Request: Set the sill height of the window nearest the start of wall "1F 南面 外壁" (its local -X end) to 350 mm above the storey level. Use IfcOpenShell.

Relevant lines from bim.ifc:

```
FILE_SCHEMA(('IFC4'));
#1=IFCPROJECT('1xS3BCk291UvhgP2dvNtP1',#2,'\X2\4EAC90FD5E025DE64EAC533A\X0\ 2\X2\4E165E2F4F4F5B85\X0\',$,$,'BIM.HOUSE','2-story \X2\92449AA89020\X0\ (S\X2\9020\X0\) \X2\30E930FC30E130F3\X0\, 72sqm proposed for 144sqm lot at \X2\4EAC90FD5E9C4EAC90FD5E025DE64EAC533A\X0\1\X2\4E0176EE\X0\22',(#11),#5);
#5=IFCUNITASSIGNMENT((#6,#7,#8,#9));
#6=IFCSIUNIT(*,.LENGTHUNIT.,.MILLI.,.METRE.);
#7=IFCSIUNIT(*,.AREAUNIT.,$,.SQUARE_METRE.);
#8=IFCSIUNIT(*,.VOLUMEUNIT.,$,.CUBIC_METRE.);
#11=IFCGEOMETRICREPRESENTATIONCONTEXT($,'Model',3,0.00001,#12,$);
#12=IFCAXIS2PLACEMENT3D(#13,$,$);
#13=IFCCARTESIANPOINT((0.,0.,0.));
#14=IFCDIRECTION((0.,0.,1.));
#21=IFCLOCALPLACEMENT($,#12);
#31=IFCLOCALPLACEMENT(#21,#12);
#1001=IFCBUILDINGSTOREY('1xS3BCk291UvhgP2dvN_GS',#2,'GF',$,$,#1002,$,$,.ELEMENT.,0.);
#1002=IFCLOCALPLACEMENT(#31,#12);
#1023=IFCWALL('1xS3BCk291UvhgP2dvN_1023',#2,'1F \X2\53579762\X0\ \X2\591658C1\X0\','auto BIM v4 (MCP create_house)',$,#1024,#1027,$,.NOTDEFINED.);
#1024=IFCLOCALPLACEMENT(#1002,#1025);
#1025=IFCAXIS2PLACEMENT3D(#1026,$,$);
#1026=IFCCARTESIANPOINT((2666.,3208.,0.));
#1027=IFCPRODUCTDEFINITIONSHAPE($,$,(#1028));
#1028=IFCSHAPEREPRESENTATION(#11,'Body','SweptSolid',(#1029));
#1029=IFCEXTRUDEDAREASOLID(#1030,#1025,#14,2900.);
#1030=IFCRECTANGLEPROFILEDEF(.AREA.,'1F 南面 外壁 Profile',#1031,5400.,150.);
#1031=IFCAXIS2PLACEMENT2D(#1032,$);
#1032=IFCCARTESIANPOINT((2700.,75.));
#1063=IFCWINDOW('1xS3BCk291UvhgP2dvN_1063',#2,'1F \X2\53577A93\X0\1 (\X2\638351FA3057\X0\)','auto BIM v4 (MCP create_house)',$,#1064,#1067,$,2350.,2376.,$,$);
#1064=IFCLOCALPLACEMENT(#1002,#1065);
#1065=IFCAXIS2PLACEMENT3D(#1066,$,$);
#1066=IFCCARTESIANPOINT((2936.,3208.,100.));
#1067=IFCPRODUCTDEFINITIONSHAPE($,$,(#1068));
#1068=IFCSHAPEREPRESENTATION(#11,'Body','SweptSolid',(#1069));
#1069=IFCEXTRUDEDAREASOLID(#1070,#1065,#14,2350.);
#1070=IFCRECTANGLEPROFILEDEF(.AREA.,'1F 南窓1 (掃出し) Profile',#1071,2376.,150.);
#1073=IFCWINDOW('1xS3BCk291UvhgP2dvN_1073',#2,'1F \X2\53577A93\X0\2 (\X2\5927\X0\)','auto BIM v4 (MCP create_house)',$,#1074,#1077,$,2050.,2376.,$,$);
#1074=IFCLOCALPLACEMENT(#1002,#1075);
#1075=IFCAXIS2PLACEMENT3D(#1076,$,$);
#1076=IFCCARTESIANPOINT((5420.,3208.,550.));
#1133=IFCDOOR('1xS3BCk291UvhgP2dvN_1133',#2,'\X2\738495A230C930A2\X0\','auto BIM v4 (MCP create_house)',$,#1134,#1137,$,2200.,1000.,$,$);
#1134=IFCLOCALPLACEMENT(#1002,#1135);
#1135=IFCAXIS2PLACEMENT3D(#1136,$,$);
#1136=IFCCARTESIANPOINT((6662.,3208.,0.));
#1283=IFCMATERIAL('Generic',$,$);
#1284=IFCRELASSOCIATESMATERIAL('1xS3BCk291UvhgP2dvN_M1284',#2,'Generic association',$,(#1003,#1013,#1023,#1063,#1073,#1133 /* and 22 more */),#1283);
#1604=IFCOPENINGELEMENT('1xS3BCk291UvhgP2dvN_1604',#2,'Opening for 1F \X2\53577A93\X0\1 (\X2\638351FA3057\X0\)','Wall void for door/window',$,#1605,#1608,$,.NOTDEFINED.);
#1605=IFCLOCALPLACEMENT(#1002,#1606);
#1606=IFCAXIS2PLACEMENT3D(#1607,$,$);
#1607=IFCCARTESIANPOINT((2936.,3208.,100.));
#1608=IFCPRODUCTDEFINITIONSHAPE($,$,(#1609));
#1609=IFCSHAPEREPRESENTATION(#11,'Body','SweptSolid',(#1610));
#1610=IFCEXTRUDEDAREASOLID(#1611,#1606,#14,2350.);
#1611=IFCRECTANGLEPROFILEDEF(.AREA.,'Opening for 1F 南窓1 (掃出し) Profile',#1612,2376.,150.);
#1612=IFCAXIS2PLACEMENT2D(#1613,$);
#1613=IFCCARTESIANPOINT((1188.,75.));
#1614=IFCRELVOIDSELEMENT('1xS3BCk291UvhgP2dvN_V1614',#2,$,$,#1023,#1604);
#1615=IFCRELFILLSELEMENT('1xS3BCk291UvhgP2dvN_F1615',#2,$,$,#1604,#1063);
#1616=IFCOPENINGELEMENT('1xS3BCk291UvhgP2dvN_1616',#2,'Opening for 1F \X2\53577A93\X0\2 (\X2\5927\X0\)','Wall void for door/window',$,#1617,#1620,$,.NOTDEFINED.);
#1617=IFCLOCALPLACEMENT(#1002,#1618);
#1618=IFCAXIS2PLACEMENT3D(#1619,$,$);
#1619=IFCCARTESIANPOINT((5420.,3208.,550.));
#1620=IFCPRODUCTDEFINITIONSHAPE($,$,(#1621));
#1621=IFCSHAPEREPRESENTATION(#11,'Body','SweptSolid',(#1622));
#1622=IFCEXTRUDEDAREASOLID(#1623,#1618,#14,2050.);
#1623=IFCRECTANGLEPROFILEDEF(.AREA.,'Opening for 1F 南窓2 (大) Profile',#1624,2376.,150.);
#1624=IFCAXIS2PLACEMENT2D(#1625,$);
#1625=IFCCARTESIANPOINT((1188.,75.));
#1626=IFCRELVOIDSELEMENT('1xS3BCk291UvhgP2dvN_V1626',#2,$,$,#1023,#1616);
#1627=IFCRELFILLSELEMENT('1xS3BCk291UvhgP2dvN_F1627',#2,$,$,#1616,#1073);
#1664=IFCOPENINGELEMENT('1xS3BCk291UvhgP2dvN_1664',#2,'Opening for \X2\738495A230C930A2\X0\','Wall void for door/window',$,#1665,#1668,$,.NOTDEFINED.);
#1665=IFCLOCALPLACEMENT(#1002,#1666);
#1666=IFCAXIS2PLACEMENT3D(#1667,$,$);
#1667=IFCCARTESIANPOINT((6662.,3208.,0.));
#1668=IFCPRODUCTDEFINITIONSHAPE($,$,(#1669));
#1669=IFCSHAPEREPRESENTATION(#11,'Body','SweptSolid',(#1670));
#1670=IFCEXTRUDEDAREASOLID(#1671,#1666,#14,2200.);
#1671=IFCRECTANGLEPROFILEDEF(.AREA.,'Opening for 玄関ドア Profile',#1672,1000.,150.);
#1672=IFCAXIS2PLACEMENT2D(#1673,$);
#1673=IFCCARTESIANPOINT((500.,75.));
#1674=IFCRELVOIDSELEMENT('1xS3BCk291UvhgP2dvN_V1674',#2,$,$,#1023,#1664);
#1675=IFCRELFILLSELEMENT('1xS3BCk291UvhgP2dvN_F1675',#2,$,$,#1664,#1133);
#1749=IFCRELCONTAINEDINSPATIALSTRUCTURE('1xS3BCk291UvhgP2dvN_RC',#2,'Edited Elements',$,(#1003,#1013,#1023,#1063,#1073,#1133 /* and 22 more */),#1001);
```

```python
import numpy as np
import ifcopenshell
import ifcopenshell.api.geometry
import ifcopenshell.geom
import ifcopenshell.util.element
import ifcopenshell.util.placement
import ifcopenshell.util.shape
import ifcopenshell.util.unit

model = ifcopenshell.open("bim.ifc")
unit_scale = ifcopenshell.util.unit.calculate_unit_scale(model)

window = model.by_guid("1xS3BCk291UvhgP2dvN_1063")
opening = window.FillsVoids[0].RelatingOpeningElement
storey = ifcopenshell.util.element.get_container(window, ifc_class="IfcBuildingStorey")
level = ifcopenshell.util.placement.get_local_placement(storey.ObjectPlacement)[2, 3]

# The opening's origin need not be at the sill, so measure its lowest point.
shape = ifcopenshell.geom.create_shape(ifcopenshell.geom.settings(), opening)
bottom = ifcopenshell.util.shape.get_shape_bottom_elevation(shape, shape.geometry) / unit_scale
dz = level + 0.35 / unit_scale - bottom

shift = np.array([0.0, 0.0, dz])
# The window is not placed relative to its opening, so move both.
for product in (opening, window):
    matrix = ifcopenshell.util.placement.get_local_placement(product.ObjectPlacement)
    matrix[:3, 3] += shift
    ifcopenshell.api.geometry.edit_object_placement(model, product=product, matrix=matrix, is_si=False)

print(f"moved by {dz * unit_scale:+.3f} m")

model.write("bim_updated.ifc")
```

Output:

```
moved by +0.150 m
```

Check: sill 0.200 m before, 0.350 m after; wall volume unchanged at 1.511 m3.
